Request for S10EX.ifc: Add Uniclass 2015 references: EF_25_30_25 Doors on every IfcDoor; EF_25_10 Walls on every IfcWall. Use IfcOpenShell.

First a look at what the model holds.

```python
import ifcopenshell

model = ifcopenshell.open("S10EX.ifc")
print(model.schema)
print("classifications:", [c.Name for c in model.by_type("IfcClassification")])
for ifc_class in ("IfcDoor", "IfcRoof", "IfcStair", "IfcWall", "IfcWindow"):
    print(ifc_class, len(model.by_type(ifc_class)))
```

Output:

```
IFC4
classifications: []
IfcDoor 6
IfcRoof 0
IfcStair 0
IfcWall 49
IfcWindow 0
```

```python
import ifcopenshell
import ifcopenshell.api.classification

model = ifcopenshell.open("S10EX.ifc")

system = ifcopenshell.api.classification.add_classification(model, classification="Uniclass 2015")

codes = {
    "IfcDoor": ("EF_25_30_25", "Doors"),
    "IfcWall": ("EF_25_10", "Walls"),
}
for ifc_class, (code, name) in codes.items():
    products = model.by_type(ifc_class)
    ifcopenshell.api.classification.add_reference(
        model, products=products, classification=system, identification=code, name=name
    )
    print(code, len(products))

model.write("S10EX_edited.ifc")
```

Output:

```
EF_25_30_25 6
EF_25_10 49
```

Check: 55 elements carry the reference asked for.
